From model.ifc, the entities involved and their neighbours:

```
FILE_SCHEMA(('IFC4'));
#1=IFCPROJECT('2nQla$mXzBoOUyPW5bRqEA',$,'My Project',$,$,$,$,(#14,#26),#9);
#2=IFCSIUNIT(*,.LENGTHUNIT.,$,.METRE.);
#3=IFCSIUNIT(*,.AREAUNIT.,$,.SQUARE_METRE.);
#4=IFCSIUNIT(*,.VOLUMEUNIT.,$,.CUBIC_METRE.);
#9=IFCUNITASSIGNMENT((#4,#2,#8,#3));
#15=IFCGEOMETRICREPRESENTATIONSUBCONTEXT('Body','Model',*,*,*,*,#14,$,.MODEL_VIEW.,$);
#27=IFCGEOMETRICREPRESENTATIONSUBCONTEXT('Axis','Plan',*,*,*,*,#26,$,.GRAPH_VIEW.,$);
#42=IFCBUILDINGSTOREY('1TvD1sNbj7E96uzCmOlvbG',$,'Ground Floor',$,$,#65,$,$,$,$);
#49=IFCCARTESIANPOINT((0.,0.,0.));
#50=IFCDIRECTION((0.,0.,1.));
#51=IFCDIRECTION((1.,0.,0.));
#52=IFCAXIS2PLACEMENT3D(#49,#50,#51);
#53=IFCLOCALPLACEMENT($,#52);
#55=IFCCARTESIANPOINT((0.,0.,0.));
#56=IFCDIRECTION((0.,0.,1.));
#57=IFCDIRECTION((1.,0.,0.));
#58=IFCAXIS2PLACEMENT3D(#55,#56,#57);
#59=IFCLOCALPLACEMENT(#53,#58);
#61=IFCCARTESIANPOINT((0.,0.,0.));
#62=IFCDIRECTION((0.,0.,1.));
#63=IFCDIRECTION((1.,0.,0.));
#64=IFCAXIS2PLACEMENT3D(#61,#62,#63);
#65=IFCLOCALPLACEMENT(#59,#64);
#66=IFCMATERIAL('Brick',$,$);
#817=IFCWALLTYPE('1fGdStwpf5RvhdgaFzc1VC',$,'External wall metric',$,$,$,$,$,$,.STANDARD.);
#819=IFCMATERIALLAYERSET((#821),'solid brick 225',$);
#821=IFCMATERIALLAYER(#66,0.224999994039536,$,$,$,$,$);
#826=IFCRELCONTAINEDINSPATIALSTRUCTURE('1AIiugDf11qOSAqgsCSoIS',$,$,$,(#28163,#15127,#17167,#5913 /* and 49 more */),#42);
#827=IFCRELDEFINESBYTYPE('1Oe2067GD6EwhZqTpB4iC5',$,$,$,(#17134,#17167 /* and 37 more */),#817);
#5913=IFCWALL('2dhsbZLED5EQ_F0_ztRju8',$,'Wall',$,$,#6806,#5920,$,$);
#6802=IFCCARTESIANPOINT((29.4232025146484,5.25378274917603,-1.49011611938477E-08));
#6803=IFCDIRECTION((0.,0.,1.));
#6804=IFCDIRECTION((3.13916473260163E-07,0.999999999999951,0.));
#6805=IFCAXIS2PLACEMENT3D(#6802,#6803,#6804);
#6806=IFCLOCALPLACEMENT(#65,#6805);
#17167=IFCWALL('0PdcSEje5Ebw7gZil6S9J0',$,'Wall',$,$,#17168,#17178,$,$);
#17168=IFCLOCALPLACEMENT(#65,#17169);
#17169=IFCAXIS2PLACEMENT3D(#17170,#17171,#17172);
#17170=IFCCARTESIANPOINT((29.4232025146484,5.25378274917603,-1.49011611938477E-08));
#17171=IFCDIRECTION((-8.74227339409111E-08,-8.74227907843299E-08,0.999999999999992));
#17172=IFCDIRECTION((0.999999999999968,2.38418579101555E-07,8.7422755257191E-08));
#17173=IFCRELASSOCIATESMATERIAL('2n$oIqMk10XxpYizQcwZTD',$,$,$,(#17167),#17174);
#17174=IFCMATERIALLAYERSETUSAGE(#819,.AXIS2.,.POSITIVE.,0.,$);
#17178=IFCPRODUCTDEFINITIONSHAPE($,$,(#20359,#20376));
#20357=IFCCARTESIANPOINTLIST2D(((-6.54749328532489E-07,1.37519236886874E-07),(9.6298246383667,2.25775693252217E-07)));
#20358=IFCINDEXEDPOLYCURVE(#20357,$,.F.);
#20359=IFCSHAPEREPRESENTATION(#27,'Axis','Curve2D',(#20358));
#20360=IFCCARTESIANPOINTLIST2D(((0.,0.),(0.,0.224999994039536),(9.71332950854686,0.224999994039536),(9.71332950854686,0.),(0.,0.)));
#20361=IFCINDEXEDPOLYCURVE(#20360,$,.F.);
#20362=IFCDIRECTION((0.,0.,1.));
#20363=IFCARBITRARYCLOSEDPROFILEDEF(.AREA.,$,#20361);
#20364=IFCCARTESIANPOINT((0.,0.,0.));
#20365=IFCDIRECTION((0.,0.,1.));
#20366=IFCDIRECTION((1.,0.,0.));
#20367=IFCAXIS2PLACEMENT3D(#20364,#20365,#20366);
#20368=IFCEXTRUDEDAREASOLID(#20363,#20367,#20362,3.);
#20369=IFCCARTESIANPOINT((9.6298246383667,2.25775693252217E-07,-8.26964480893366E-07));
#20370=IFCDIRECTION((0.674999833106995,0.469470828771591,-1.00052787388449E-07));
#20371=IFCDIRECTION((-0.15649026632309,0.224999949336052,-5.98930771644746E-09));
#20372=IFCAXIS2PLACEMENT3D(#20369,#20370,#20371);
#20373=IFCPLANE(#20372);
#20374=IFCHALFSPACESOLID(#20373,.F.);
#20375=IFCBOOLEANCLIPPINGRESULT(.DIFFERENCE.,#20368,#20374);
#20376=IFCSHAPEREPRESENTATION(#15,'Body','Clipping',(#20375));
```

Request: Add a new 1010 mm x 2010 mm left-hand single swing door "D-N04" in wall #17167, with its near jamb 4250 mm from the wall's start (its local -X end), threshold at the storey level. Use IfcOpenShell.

```python
import numpy as np
import ifcopenshell
import ifcopenshell.api.feature
import ifcopenshell.api.geometry
import ifcopenshell.api.root
import ifcopenshell.api.spatial
import ifcopenshell.geom
import ifcopenshell.util.element
import ifcopenshell.util.placement
import ifcopenshell.util.representation
import ifcopenshell.util.shape
import ifcopenshell.util.unit

model = ifcopenshell.open("model.ifc")
unit_scale = ifcopenshell.util.unit.calculate_unit_scale(model)
settings = ifcopenshell.geom.settings()


def volume(element):
    """Net volume in cubic metres, openings subtracted."""
    shape = ifcopenshell.geom.create_shape(settings, element)
    return ifcopenshell.util.shape.get_volume(shape.geometry)


wall = model.by_guid("0PdcSEje5Ebw7gZil6S9J0")
storey = ifcopenshell.util.element.get_container(wall, ifc_class="IfcBuildingStorey")
context = ifcopenshell.util.representation.get_context(model, "Model", "Body", "MODEL_VIEW")
before = volume(wall)

width, height, from_end, sill = 1.01, 2.01, 4.25, 0.0  # metres

# The wall runs along its own X axis, and the end named is its -X end.
wall_shape = ifcopenshell.geom.create_shape(settings, wall)
x, y, z = ifcopenshell.util.shape.get_vertices(wall_shape.geometry).T
start = x.min() + from_end
face, thickness = float(y.min()), float(y.max() - y.min())
wall_matrix = ifcopenshell.util.placement.get_local_placement(wall.ObjectPlacement)
level = ifcopenshell.util.placement.get_local_placement(storey.ObjectPlacement)[2, 3]


def in_wall(x, y):
    """Placement at x, y metres in the wall's axes, at sill height."""
    matrix = wall_matrix.copy()
    matrix[:, 3] = wall_matrix @ np.array([x / unit_scale, y / unit_scale, 0.0, 1.0])
    matrix[2, 3] = level + sill / unit_scale
    return matrix


# Opening: a box that overshoots both wall faces by 50 mm.
opening = ifcopenshell.api.root.create_entity(model, ifc_class="IfcOpeningElement", predefined_type="OPENING")
box = ifcopenshell.api.geometry.add_wall_representation(
    model, context=context, length=width, height=height, thickness=thickness + 0.1
)
ifcopenshell.api.geometry.assign_representation(model, product=opening, representation=box)
ifcopenshell.api.geometry.edit_object_placement(model, product=opening, matrix=in_wall(start, face - 0.05), is_si=False)
ifcopenshell.api.feature.add_feature(model, feature=opening, element=wall)

door = ifcopenshell.api.root.create_entity(model, ifc_class="IfcDoor", name="D-N04", predefined_type="DOOR")
door.OverallWidth, door.OverallHeight = width / unit_scale, height / unit_scale
door.OperationType = "SINGLE_SWING_LEFT"
body = ifcopenshell.api.geometry.add_door_representation(
    model,
    context=context,
    overall_width=door.OverallWidth,
    overall_height=door.OverallHeight,
    operation_type="SINGLE_SWING_LEFT",
    lining_properties={"LiningDepth": thickness / unit_scale, "ThresholdDepth": thickness / unit_scale},
)
ifcopenshell.api.geometry.assign_representation(model, product=door, representation=body)
ifcopenshell.api.spatial.assign_container(model, products=[door], relating_structure=storey)
ifcopenshell.api.feature.add_filling(model, opening=opening, element=door)

# The lining spans the wall, so the door starts at the wall face.
ifcopenshell.api.geometry.edit_object_placement(model, product=door, matrix=in_wall(start, face), is_si=False)

after = volume(wall)

print(f"wall volume {before:.3f} -> {after:.3f} m3")

model.write("model-out.ifc")
```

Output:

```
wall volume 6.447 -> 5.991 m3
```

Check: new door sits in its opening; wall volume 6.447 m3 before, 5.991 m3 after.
